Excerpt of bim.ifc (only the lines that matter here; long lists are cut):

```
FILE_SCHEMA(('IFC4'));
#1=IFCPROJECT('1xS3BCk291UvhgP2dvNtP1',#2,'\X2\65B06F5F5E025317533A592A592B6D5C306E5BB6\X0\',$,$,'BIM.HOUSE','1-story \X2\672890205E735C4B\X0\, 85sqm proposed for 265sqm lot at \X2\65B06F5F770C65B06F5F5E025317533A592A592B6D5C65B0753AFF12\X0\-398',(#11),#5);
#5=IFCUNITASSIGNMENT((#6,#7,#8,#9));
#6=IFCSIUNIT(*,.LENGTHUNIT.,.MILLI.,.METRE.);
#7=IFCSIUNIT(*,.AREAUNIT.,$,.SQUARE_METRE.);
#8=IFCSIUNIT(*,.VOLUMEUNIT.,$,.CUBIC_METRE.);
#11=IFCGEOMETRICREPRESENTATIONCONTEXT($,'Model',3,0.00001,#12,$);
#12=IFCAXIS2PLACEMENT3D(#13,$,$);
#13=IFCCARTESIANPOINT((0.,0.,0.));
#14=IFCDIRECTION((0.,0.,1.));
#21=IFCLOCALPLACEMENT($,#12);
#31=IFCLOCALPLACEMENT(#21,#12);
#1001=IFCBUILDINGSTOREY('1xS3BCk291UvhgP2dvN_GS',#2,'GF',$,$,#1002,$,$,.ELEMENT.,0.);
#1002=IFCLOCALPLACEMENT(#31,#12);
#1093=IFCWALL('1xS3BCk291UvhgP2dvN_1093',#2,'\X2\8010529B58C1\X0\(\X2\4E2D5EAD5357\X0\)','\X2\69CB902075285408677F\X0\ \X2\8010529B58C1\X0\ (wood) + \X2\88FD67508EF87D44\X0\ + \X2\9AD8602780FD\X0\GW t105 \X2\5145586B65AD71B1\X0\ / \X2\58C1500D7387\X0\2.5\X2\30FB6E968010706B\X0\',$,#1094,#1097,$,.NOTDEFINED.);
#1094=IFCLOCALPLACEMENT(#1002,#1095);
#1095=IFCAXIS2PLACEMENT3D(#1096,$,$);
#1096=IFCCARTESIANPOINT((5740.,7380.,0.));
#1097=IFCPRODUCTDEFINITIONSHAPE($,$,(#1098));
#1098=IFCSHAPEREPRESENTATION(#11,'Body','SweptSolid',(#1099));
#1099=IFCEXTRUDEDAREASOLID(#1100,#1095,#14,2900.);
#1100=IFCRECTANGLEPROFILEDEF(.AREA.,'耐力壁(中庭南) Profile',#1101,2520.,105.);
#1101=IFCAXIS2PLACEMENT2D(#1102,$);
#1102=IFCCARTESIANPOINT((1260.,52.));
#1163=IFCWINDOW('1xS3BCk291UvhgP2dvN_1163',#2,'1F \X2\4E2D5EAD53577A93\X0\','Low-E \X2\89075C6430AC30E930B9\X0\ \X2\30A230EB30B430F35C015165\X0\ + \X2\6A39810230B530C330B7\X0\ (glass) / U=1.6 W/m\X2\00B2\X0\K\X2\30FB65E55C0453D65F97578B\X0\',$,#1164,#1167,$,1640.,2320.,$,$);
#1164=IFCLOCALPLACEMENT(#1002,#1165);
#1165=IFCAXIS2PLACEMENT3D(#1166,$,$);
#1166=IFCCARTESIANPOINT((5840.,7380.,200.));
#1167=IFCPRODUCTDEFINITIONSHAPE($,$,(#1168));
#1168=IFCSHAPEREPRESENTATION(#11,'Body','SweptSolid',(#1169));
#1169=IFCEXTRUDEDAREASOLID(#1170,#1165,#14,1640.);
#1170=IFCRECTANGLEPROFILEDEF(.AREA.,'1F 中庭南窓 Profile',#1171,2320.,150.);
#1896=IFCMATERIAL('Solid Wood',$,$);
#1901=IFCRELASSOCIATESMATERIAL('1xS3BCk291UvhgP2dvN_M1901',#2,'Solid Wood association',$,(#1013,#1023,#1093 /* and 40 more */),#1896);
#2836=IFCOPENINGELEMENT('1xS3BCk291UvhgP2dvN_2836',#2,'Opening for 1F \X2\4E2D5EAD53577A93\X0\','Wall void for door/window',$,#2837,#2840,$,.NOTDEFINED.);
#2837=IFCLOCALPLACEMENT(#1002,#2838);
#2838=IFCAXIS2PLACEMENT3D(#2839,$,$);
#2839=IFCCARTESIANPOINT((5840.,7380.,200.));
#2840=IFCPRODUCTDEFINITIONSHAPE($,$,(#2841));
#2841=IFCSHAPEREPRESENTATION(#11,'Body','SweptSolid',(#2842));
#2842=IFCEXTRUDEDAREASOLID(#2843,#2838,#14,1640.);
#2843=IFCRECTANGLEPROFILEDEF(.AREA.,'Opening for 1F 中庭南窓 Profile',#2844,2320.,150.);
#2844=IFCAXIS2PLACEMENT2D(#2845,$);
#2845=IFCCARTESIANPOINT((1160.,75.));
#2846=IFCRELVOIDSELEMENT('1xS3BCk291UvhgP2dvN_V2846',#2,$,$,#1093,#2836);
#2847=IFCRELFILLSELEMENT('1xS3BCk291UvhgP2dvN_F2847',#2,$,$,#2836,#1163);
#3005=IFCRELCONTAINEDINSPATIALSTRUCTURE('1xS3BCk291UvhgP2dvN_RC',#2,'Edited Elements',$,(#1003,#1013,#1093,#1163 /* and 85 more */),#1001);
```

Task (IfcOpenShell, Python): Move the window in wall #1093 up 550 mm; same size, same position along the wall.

```python
import numpy as np
import ifcopenshell
import ifcopenshell.api.geometry
import ifcopenshell.util.placement
import ifcopenshell.util.unit

model = ifcopenshell.open("bim.ifc")
unit_scale = ifcopenshell.util.unit.calculate_unit_scale(model)

window = model.by_guid("1xS3BCk291UvhgP2dvN_1163")
opening = window.FillsVoids[0].RelatingOpeningElement
dz = 0.55 / unit_scale

shift = np.array([0.0, 0.0, dz])
# The window is not placed relative to its opening, so move both.
for product in (opening, window):
    matrix = ifcopenshell.util.placement.get_local_placement(product.ObjectPlacement)
    matrix[:3, 3] += shift
    ifcopenshell.api.geometry.edit_object_placement(model, product=product, matrix=matrix, is_si=False)

print(f"moved by {dz * unit_scale:+.3f} m")

model.write("bim_v2.ifc")
```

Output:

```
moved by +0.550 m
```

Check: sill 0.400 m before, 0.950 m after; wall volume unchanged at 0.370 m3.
